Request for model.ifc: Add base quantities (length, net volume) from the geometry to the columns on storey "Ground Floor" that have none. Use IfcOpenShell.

First a look at what the model holds.

```python
import ifcopenshell
import ifcopenshell.util.element
import ifcopenshell.util.unit

model = ifcopenshell.open("model.ifc")
print(model.schema)
for unit_type in ("LENGTHUNIT", "AREAUNIT", "VOLUMEUNIT"):
    print(unit_type, ifcopenshell.util.unit.calculate_unit_scale(model, unit_type))
storey = next(s for s in model.by_type("IfcBuildingStorey") if s.Name == "Ground Floor")
columns = [e for e in ifcopenshell.util.element.get_decomposition(storey) if e.is_a("IfcColumn")]
for e in sorted(columns, key=lambda e: e.id()):
    print(e.id(), e.is_a(), e.Name, list(ifcopenshell.util.element.get_psets(e, qtos_only=True)), sep=" | ")
```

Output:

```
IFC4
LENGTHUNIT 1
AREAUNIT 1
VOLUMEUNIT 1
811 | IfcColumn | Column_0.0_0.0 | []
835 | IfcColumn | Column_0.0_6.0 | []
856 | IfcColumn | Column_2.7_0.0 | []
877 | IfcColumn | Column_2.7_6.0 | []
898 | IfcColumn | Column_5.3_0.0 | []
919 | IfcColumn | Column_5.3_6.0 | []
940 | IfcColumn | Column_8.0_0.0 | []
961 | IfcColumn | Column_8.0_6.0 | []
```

```python
import ifcopenshell
import ifcopenshell.api.pset
import ifcopenshell.geom
import ifcopenshell.util.element
import ifcopenshell.util.shape
import ifcopenshell.util.unit

model = ifcopenshell.open("model.ifc")
unit_scale = ifcopenshell.util.unit.calculate_unit_scale(model)
volume_scale = ifcopenshell.util.unit.calculate_unit_scale(model, "VOLUMEUNIT")
settings = ifcopenshell.geom.settings()

storey = next(s for s in model.by_type("IfcBuildingStorey") if s.Name == "Ground Floor")
columns = [e for e in ifcopenshell.util.element.get_decomposition(storey) if e.is_a("IfcColumn")]

for e in sorted(columns, key=lambda e: e.id()):
    if ifcopenshell.util.element.get_psets(e, qtos_only=True, should_inherit=False):
        continue
    # Geometry comes back in metres, in the element's own axes.
    shape = ifcopenshell.geom.create_shape(settings, e)
    values = {
        "Length": ifcopenshell.util.shape.get_z(shape.geometry) / unit_scale,
        "NetVolume": ifcopenshell.util.shape.get_volume(shape.geometry) / volume_scale,
    }
    qto = ifcopenshell.api.pset.add_qto(model, product=e, name="Qto_ColumnBaseQuantities")
    ifcopenshell.api.pset.edit_qto(model, qto=qto, properties=values)
    print(e.id(), {k: round(v, 3) for k, v in values.items()})

model.write("model_updated.ifc")
```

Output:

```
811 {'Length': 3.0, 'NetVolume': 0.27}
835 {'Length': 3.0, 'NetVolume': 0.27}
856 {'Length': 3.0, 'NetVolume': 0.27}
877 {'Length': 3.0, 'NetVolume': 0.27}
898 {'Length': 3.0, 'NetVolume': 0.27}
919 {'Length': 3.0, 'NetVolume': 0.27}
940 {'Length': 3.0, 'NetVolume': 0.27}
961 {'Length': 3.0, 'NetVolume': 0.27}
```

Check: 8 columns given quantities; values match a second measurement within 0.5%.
